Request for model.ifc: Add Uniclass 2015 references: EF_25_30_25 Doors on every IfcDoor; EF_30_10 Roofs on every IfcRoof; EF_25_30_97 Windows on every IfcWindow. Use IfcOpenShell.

First a look at what the model holds.

```python
import ifcopenshell

model = ifcopenshell.open("model.ifc")
print(model.schema)
print("classifications:", [c.Name for c in model.by_type("IfcClassification")])
for ifc_class in ("IfcDoor", "IfcRoof", "IfcStair", "IfcWall", "IfcWindow"):
    print(ifc_class, len(model.by_type(ifc_class)))
```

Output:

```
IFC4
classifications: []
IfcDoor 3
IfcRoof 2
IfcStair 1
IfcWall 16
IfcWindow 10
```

```python
import ifcopenshell
import ifcopenshell.api.classification

model = ifcopenshell.open("model.ifc")

system = ifcopenshell.api.classification.add_classification(model, classification="Uniclass 2015")

codes = {
    "IfcDoor": ("EF_25_30_25", "Doors"),
    "IfcRoof": ("EF_30_10", "Roofs"),
    "IfcWindow": ("EF_25_30_97", "Windows"),
}
for ifc_class, (code, name) in codes.items():
    products = model.by_type(ifc_class)
    ifcopenshell.api.classification.add_reference(
        model, products=products, classification=system, identification=code, name=name
    )
    print(code, len(products))

model.write("model_updated.ifc")
```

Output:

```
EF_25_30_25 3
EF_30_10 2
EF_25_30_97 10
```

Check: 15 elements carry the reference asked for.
